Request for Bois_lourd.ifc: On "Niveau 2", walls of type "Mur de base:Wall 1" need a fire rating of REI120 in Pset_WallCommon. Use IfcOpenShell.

First a look at what the model holds.

```python
import ifcopenshell
import ifcopenshell.util.element

model = ifcopenshell.open("Bois_lourd.ifc")
print(model.schema)
storey = next(s for s in model.by_type("IfcBuildingStorey") if s.Name == "Niveau 2")
walls = [e for e in ifcopenshell.util.element.get_decomposition(storey) if e.is_a("IfcWall")]
seen = {}
for e in walls:
    element_type = ifcopenshell.util.element.get_type(e)
    key = (element_type.Name if element_type != e and element_type else None, ifcopenshell.util.element.get_pset(e, "Pset_WallCommon", "FireRating"))
    seen[key] = seen.get(key, 0) + 1
for (name, value), count in sorted(seen.items(), key=str):
    print(count, "x", name, "|", value)
```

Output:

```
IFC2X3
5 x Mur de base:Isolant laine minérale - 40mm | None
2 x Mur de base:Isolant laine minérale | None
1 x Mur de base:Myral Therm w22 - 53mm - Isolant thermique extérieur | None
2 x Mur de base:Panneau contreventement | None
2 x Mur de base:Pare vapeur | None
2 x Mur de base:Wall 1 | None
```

```python
import ifcopenshell
import ifcopenshell.api.pset
import ifcopenshell.util.element

model = ifcopenshell.open("Bois_lourd.ifc")

storey = next(s for s in model.by_type("IfcBuildingStorey") if s.Name == "Niveau 2")
walls = [e for e in ifcopenshell.util.element.get_decomposition(storey) if e.is_a("IfcWall")]

count = 0
for e in walls:
    element_type = ifcopenshell.util.element.get_type(e)
    if element_type in (None, e) or element_type.Name != "Mur de base:Wall 1":
        continue
    # add_pset returns the element's existing set when there is one.
    pset = ifcopenshell.api.pset.add_pset(model, product=e, name="Pset_WallCommon")
    ifcopenshell.api.pset.edit_pset(model, pset=pset, properties={"FireRating": "REI120"})
    count += 1

print(count, "walls updated")

model.write("Bois_lourd_rev.ifc")
```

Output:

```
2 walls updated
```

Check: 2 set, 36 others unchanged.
